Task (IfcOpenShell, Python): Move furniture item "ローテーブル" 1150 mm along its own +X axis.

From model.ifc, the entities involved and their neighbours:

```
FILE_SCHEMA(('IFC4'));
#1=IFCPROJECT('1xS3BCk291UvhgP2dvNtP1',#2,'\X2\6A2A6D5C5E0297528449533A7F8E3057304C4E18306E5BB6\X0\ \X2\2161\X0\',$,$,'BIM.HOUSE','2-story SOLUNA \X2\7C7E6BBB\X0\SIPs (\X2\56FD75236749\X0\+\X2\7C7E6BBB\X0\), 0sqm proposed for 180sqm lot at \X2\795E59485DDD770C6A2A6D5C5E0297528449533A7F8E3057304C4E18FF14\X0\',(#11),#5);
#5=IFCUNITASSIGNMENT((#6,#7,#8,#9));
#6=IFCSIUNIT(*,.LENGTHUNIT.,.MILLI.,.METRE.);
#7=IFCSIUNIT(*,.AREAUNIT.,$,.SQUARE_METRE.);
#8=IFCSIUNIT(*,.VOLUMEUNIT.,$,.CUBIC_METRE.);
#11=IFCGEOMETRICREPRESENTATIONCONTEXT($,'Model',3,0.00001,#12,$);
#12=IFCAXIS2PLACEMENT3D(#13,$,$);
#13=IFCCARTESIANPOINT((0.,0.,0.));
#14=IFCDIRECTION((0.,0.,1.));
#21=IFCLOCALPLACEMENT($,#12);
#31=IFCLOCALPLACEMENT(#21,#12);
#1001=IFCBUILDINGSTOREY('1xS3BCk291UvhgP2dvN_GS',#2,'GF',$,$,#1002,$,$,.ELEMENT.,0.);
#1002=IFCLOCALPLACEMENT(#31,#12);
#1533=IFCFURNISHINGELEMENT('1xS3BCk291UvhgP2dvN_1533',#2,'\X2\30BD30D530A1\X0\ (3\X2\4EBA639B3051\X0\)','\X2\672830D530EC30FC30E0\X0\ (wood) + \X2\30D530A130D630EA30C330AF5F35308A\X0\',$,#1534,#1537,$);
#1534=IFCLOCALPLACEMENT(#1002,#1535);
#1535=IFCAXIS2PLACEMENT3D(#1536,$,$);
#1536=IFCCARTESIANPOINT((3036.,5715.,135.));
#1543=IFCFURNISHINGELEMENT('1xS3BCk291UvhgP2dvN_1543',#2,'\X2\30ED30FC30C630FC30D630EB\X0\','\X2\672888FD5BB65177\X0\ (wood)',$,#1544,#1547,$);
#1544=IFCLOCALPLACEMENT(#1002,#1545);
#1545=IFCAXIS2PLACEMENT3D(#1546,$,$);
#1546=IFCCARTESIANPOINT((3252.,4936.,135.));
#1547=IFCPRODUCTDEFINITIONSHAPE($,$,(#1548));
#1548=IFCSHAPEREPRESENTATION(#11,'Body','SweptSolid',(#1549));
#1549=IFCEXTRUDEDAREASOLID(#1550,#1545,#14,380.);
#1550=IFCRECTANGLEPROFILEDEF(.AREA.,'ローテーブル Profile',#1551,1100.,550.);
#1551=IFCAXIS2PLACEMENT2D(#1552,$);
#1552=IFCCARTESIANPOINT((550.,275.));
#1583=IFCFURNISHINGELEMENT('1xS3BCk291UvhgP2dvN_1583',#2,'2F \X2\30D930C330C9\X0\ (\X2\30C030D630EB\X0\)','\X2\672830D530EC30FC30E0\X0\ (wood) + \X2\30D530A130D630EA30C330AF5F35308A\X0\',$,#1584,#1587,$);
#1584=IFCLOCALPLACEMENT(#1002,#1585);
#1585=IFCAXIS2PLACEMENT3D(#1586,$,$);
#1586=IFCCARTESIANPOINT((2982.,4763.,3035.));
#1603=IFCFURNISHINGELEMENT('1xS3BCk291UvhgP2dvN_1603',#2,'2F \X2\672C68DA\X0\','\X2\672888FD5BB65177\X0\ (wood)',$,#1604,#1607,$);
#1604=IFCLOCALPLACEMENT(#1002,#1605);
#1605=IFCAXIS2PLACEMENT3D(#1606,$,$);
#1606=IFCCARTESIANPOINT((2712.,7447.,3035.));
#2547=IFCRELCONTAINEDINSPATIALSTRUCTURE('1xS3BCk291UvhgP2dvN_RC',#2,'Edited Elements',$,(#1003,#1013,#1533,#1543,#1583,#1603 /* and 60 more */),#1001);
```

```python
import ifcopenshell
import ifcopenshell.api.geometry
import ifcopenshell.util.placement
import ifcopenshell.util.unit

model = ifcopenshell.open("model.ifc")
unit_scale = ifcopenshell.util.unit.calculate_unit_scale(model)

item = model.by_guid("1xS3BCk291UvhgP2dvN_1543")
matrix = ifcopenshell.util.placement.get_local_placement(item.ObjectPlacement)
matrix[:3, 3] += matrix[:3, 0] * 1.15 / unit_scale
ifcopenshell.api.geometry.edit_object_placement(model, product=item, matrix=matrix, is_si=False)

print(ifcopenshell.util.placement.get_local_placement(item.ObjectPlacement).round(3) + 0.0)

model.write("model_updated.ifc")
```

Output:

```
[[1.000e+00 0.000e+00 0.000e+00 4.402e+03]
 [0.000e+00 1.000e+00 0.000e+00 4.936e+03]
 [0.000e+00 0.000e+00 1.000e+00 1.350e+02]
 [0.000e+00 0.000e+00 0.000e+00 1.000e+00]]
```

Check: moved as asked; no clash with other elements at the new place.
